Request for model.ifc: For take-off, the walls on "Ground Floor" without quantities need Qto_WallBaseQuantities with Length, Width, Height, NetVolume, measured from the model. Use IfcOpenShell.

First a look at what the model holds.

```python
import ifcopenshell
import ifcopenshell.util.element
import ifcopenshell.util.unit

model = ifcopenshell.open("model.ifc")
print(model.schema)
for unit_type in ("LENGTHUNIT", "AREAUNIT", "VOLUMEUNIT"):
    print(unit_type, ifcopenshell.util.unit.calculate_unit_scale(model, unit_type))
storey = next(s for s in model.by_type("IfcBuildingStorey") if s.Name == "Ground Floor")
walls = [e for e in ifcopenshell.util.element.get_decomposition(storey) if e.is_a("IfcWall")]
for e in sorted(walls, key=lambda e: e.id()):
    print(e.id(), e.is_a(), e.Name, list(ifcopenshell.util.element.get_psets(e, qtos_only=True)), sep=" | ")
```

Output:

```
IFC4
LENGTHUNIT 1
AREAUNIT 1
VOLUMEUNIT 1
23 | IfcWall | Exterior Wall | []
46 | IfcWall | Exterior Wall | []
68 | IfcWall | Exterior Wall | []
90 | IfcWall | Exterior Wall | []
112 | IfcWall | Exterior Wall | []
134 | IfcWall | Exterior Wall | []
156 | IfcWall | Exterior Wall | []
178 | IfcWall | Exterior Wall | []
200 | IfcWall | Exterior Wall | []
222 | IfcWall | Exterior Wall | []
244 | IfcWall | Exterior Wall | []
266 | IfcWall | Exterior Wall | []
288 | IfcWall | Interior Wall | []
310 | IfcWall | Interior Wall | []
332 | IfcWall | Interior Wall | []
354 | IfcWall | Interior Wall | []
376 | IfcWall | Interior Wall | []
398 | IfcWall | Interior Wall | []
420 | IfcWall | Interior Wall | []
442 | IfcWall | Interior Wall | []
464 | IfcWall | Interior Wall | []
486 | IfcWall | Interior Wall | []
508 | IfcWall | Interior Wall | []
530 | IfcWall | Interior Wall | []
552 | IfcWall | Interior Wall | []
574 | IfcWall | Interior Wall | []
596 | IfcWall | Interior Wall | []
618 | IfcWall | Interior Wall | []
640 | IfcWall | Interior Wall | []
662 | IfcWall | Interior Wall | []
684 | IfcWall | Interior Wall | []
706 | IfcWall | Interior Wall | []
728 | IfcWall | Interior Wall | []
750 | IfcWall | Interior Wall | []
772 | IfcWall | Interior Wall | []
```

```python
import ifcopenshell
import ifcopenshell.api.pset
import ifcopenshell.geom
import ifcopenshell.util.element
import ifcopenshell.util.shape
import ifcopenshell.util.unit

model = ifcopenshell.open("model.ifc")
unit_scale = ifcopenshell.util.unit.calculate_unit_scale(model)
volume_scale = ifcopenshell.util.unit.calculate_unit_scale(model, "VOLUMEUNIT")
settings = ifcopenshell.geom.settings()

storey = next(s for s in model.by_type("IfcBuildingStorey") if s.Name == "Ground Floor")
walls = [e for e in ifcopenshell.util.element.get_decomposition(storey) if e.is_a("IfcWall")]

for e in sorted(walls, key=lambda e: e.id()):
    if ifcopenshell.util.element.get_psets(e, qtos_only=True, should_inherit=False):
        continue
    # Geometry comes back in metres, in the element's own axes.
    shape = ifcopenshell.geom.create_shape(settings, e)
    values = {
        "Length": ifcopenshell.util.shape.get_x(shape.geometry) / unit_scale,
        "Width": ifcopenshell.util.shape.get_y(shape.geometry) / unit_scale,
        "Height": ifcopenshell.util.shape.get_z(shape.geometry) / unit_scale,
        "NetVolume": ifcopenshell.util.shape.get_volume(shape.geometry) / volume_scale,
    }
    qto = ifcopenshell.api.pset.add_qto(model, product=e, name="Qto_WallBaseQuantities")
    ifcopenshell.api.pset.edit_qto(model, qto=qto, properties=values)
    print(e.id(), {k: round(v, 3) for k, v in values.items()})

model.write("model_v2.ifc")
```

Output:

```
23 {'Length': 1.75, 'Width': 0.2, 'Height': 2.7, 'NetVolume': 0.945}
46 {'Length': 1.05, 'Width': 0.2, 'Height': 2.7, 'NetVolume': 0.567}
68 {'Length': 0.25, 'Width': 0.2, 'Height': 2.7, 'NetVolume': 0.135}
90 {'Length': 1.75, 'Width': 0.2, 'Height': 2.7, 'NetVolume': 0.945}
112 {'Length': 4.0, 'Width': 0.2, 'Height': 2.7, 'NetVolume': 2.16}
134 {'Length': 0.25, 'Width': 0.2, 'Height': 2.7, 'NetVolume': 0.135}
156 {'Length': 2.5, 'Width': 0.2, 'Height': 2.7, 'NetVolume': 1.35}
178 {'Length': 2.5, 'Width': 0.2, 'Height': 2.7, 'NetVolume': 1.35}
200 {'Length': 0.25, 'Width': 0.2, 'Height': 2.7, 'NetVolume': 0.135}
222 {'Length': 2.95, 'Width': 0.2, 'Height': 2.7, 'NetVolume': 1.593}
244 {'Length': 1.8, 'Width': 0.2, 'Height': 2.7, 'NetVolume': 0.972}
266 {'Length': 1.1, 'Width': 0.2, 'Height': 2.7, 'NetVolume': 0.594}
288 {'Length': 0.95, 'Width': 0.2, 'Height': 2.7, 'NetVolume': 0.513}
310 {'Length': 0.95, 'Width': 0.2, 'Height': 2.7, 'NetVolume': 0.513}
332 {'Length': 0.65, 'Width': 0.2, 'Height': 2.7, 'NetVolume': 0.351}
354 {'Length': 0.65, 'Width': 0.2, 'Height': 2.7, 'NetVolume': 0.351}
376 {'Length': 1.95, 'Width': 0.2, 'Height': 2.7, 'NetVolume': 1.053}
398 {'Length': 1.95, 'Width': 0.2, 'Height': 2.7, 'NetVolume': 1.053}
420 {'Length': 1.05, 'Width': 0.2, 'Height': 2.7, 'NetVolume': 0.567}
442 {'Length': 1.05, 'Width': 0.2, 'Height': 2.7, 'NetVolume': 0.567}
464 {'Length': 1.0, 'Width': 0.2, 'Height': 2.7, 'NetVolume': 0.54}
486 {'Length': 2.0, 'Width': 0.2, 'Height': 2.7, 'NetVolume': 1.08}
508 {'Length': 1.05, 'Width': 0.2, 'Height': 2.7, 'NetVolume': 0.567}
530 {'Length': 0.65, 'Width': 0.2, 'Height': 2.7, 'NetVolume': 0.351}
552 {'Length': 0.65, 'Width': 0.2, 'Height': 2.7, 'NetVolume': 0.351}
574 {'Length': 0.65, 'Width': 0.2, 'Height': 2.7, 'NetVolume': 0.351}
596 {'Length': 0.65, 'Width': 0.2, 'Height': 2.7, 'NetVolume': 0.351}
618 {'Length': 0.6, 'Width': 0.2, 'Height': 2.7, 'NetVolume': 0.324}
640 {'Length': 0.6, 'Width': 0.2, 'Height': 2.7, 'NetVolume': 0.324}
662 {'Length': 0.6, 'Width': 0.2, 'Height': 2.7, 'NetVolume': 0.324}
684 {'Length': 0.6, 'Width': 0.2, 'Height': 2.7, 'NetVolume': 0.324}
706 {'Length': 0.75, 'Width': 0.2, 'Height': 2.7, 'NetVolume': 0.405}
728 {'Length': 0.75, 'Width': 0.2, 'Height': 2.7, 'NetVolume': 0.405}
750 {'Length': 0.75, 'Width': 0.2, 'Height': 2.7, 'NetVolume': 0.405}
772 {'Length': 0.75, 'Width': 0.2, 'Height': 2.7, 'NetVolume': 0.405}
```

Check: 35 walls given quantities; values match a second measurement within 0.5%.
